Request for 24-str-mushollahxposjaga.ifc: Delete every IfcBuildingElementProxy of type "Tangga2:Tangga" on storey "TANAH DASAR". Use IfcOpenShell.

First a look at what the model holds.

```python
import ifcopenshell
import ifcopenshell.util.element

model = ifcopenshell.open("24-str-mushollahxposjaga.ifc")
print(model.schema)
storey = next(s for s in model.by_type("IfcBuildingStorey") if s.Name == "TANAH DASAR")
proxies = [e for e in ifcopenshell.util.element.get_decomposition(storey) if e.is_a("IfcBuildingElementProxy")]
seen = {}
for e in proxies:
    element_type = ifcopenshell.util.element.get_type(e)
    name = element_type.Name if element_type not in (None, e) else None
    seen[name] = seen.get(name, 0) + 1
for name, count in sorted(seen.items(), key=str):
    print(count, "x", name)
```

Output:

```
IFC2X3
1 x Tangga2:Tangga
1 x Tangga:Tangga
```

```python
import ifcopenshell
import ifcopenshell.api.root
import ifcopenshell.util.element

model = ifcopenshell.open("24-str-mushollahxposjaga.ifc")

storey = next(s for s in model.by_type("IfcBuildingStorey") if s.Name == "TANAH DASAR")
proxies = [e for e in ifcopenshell.util.element.get_decomposition(storey) if e.is_a("IfcBuildingElementProxy")]
targets = [e for e in proxies if (t := ifcopenshell.util.element.get_type(e)) not in (None, e) and t.Name == "Tangga2:Tangga"]

for e in targets:
    ifcopenshell.api.root.remove_product(model, product=e)
print(len(targets), "removed")

model.write("24-str-mushollahxposjaga_v2.ifc")
```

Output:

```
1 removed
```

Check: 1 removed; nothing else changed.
